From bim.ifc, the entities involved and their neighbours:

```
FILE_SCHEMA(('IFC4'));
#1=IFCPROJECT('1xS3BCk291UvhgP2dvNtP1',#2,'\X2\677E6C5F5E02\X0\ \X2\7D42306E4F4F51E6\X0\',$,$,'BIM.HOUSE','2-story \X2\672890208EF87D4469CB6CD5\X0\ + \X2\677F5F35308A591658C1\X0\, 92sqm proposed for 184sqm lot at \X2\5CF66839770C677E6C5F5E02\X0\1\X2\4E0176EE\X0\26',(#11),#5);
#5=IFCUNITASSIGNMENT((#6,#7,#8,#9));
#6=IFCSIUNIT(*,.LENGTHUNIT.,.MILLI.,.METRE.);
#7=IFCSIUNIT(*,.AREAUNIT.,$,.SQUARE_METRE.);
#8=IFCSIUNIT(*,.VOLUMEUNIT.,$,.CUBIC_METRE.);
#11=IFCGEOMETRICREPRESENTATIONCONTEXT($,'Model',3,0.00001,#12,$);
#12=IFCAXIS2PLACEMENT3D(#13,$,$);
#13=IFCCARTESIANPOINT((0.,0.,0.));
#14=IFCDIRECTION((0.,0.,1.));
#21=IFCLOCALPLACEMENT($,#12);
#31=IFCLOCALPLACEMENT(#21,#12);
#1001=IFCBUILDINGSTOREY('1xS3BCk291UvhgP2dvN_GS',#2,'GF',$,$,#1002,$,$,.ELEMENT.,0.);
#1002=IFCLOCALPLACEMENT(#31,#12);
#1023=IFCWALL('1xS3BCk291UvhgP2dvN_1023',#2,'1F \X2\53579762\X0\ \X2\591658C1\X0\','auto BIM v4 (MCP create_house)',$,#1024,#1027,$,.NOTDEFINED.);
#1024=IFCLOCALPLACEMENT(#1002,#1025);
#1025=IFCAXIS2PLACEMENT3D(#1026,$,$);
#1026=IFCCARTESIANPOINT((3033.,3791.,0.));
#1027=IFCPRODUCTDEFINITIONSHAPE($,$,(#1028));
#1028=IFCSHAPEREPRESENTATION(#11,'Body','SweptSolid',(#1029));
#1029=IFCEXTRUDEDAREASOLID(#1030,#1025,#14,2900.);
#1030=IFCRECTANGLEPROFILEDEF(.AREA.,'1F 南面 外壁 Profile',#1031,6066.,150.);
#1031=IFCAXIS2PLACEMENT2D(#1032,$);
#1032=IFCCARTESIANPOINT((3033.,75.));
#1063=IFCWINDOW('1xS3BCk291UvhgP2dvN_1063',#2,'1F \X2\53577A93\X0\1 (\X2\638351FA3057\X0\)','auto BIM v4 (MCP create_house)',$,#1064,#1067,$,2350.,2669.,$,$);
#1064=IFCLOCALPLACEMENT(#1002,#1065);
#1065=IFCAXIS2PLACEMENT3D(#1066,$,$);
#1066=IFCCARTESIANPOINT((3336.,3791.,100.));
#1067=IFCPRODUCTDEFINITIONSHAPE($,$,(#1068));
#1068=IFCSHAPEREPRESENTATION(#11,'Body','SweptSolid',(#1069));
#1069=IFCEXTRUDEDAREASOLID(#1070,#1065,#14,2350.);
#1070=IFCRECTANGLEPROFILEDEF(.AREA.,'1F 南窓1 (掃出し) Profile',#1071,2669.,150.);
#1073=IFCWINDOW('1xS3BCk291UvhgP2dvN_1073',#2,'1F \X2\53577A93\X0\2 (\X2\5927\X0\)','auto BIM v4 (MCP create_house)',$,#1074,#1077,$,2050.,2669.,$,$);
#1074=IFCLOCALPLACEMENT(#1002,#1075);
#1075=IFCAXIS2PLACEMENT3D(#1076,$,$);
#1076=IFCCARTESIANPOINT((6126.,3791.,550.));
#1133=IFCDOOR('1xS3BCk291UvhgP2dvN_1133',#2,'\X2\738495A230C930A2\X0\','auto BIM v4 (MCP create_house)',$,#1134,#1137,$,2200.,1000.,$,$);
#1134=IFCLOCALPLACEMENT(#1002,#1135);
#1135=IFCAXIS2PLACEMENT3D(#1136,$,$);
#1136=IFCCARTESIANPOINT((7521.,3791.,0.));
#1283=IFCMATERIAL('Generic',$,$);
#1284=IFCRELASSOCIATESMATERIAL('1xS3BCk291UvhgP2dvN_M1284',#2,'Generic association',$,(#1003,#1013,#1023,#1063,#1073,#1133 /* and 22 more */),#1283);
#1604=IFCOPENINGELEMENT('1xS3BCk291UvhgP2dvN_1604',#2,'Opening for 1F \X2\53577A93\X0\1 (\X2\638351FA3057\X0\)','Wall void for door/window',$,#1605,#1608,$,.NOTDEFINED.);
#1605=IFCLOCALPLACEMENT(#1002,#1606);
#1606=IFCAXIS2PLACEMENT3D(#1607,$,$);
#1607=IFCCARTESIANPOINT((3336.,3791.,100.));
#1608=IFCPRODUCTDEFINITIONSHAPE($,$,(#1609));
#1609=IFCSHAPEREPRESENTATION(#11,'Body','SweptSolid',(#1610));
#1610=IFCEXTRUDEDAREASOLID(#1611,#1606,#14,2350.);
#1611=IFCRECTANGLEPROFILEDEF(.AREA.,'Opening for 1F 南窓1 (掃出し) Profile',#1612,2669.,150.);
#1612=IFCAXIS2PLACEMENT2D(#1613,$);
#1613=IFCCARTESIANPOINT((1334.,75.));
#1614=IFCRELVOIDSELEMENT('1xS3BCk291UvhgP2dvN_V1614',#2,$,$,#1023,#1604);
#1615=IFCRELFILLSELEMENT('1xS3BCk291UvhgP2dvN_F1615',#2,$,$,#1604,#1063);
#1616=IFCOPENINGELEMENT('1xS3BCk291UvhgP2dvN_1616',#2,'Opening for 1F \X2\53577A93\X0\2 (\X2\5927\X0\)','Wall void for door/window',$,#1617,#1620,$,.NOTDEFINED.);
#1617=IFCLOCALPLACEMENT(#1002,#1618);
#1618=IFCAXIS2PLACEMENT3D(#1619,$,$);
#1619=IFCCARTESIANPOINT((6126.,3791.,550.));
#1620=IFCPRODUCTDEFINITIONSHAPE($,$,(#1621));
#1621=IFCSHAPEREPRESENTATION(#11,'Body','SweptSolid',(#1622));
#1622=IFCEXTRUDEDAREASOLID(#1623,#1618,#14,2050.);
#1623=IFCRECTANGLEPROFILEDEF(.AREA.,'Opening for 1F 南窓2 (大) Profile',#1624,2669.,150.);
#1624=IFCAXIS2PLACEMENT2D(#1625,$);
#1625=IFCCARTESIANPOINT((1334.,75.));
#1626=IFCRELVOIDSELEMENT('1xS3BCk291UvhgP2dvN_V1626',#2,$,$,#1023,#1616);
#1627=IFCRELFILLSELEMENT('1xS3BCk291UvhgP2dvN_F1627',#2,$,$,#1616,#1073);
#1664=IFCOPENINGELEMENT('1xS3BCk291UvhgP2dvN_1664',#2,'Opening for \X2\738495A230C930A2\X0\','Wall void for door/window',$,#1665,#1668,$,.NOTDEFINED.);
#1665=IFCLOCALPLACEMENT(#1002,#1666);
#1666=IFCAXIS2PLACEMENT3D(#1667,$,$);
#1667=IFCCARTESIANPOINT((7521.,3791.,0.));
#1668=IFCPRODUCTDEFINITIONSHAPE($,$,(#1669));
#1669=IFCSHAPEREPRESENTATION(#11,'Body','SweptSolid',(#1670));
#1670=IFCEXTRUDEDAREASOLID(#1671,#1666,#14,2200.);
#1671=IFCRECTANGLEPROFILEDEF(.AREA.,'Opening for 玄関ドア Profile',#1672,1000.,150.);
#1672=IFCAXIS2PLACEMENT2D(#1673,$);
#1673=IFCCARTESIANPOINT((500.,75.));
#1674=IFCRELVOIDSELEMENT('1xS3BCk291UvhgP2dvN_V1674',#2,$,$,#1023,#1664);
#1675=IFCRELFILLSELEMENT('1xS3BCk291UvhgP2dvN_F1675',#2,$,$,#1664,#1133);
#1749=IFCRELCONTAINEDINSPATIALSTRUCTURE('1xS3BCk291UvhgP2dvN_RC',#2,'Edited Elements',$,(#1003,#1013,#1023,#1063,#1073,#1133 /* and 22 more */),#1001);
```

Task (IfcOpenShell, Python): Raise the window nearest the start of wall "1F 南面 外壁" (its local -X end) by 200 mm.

```python
import numpy as np
import ifcopenshell
import ifcopenshell.api.geometry
import ifcopenshell.util.placement
import ifcopenshell.util.unit

model = ifcopenshell.open("bim.ifc")
unit_scale = ifcopenshell.util.unit.calculate_unit_scale(model)

window = model.by_guid("1xS3BCk291UvhgP2dvN_1063")
opening = window.FillsVoids[0].RelatingOpeningElement
dz = 0.2 / unit_scale

shift = np.array([0.0, 0.0, dz])
# The window is not placed relative to its opening, so move both.
for product in (opening, window):
    matrix = ifcopenshell.util.placement.get_local_placement(product.ObjectPlacement)
    matrix[:3, 3] += shift
    ifcopenshell.api.geometry.edit_object_placement(model, product=product, matrix=matrix, is_si=False)

print(f"moved by {dz * unit_scale:+.3f} m")

model.write("bim_rev.ifc")
```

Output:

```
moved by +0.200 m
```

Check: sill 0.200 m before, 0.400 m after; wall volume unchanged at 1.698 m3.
